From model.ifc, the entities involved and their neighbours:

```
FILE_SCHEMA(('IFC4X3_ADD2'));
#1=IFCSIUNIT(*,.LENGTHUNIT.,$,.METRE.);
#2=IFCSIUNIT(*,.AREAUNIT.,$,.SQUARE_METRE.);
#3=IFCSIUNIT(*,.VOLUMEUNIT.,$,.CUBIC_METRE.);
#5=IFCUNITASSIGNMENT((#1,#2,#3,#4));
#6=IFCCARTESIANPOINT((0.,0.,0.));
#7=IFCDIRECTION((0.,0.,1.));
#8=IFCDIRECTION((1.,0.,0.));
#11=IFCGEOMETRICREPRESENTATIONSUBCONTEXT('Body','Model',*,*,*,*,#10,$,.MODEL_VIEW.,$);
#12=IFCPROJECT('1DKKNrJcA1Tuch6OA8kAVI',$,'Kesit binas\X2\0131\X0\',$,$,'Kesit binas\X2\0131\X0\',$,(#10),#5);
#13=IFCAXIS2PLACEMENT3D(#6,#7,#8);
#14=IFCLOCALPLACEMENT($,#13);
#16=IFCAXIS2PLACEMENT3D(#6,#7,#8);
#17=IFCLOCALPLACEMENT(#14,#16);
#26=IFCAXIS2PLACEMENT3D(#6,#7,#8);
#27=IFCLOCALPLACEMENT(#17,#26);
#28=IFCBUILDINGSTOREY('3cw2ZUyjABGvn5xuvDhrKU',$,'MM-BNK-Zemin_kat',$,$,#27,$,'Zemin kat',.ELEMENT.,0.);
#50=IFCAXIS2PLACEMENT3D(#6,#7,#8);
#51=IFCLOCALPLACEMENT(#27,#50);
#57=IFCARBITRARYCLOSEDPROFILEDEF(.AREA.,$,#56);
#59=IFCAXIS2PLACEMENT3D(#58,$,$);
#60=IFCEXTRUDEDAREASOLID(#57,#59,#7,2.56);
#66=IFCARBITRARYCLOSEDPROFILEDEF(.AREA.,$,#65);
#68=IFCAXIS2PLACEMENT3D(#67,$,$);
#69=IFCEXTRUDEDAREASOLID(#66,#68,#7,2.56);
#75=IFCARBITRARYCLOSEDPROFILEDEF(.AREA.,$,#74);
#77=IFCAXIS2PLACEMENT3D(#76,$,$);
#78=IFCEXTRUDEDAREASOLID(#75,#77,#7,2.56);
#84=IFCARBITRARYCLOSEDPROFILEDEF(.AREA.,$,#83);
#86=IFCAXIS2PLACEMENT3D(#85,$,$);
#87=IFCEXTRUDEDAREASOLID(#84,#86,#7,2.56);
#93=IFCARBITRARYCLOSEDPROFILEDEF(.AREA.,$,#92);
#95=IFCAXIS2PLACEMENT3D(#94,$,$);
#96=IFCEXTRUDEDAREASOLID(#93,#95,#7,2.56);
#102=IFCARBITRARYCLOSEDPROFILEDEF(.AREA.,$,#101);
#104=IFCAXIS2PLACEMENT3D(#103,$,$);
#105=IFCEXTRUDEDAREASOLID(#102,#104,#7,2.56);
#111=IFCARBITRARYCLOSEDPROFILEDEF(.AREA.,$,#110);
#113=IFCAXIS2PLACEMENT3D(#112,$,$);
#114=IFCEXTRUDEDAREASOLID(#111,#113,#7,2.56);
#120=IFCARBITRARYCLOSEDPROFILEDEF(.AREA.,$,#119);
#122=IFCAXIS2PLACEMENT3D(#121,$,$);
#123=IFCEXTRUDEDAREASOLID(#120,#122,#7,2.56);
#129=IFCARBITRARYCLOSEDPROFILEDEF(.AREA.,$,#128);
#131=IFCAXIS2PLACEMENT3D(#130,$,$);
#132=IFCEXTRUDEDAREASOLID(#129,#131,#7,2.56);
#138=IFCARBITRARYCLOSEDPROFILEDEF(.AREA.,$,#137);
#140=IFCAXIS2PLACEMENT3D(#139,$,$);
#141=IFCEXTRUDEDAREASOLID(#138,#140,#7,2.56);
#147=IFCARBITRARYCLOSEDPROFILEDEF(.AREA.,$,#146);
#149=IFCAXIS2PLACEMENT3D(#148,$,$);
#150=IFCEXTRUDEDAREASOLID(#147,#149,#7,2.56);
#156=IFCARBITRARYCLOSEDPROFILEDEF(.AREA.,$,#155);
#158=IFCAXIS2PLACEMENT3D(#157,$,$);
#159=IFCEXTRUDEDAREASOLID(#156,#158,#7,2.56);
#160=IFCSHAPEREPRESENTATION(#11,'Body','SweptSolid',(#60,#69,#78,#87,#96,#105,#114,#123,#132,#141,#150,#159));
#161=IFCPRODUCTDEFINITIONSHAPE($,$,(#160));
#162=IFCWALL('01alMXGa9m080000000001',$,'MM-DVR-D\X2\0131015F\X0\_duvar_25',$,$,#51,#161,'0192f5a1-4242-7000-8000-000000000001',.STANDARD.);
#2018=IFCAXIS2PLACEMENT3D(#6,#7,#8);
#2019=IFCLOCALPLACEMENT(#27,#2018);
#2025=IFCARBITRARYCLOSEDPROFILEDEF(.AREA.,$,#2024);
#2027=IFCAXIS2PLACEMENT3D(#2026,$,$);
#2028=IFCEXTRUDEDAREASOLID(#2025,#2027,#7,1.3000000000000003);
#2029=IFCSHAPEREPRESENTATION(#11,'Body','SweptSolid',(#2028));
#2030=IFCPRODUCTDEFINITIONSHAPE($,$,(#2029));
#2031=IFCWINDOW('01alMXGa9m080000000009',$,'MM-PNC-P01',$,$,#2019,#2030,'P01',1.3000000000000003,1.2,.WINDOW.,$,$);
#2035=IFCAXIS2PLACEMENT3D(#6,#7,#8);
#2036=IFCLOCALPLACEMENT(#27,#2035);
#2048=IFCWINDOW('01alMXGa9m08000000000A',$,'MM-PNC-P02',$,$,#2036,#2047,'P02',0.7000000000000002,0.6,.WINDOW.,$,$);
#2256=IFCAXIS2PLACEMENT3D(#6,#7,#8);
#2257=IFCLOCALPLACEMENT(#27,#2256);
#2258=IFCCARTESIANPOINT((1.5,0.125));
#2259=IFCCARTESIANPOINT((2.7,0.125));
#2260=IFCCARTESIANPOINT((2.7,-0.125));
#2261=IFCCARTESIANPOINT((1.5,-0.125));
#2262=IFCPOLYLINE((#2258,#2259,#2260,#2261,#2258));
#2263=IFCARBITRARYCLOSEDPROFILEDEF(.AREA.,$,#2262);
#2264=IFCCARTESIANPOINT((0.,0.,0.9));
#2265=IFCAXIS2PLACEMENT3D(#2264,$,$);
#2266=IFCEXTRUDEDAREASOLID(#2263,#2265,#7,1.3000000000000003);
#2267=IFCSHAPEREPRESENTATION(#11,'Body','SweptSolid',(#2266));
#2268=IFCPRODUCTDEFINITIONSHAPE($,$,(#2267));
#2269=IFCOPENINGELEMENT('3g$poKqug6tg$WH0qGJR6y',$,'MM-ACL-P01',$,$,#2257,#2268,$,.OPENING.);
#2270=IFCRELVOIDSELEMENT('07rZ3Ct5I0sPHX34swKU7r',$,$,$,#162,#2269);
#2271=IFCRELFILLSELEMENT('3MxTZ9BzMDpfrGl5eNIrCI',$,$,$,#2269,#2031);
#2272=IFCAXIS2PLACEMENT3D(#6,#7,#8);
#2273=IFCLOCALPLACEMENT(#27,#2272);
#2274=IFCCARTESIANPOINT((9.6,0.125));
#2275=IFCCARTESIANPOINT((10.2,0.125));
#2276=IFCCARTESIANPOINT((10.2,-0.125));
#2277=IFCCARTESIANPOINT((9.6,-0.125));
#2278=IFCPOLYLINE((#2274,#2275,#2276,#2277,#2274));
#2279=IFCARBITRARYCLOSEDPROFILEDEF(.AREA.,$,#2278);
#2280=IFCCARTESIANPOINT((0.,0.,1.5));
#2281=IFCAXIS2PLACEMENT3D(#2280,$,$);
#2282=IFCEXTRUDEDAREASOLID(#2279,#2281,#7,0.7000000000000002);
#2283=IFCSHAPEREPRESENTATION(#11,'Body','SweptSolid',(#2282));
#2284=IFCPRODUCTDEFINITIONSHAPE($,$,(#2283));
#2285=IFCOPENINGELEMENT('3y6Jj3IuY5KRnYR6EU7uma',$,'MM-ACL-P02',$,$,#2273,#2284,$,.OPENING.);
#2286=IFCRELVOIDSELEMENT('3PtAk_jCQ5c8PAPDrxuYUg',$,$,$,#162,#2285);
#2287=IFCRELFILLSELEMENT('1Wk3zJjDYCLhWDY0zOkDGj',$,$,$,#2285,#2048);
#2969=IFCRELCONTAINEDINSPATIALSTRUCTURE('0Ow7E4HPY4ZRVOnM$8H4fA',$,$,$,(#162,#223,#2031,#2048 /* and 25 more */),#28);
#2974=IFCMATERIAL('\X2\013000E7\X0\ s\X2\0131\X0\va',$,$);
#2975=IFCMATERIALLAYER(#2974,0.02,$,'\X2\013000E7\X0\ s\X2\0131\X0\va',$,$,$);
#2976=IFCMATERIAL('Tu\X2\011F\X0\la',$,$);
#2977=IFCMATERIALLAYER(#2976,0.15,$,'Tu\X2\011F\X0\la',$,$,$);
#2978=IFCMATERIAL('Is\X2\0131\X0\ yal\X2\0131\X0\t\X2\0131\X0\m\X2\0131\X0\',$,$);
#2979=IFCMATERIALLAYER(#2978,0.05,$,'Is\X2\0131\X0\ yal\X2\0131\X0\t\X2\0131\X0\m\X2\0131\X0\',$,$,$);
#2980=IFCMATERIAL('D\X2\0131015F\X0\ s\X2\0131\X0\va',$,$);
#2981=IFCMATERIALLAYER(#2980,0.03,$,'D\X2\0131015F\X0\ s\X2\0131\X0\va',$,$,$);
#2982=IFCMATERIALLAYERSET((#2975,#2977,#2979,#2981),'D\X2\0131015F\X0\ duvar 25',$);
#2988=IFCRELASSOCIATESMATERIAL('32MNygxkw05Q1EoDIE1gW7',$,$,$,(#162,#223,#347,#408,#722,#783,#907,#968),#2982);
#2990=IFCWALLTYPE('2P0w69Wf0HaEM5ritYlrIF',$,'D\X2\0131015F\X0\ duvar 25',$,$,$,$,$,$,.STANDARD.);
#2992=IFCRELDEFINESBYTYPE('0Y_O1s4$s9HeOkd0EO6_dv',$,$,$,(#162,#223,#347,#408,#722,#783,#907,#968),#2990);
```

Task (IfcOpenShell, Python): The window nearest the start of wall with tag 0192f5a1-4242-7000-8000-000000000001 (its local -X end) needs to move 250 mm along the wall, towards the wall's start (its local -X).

```python
import ifcopenshell
import ifcopenshell.api.geometry
import ifcopenshell.util.placement

model = ifcopenshell.open("model.ifc")

window = model.by_guid("01alMXGa9m080000000009")
opening = window.FillsVoids[0].RelatingOpeningElement
wall = opening.VoidsElements[0].RelatingBuildingElement

wall_matrix = ifcopenshell.util.placement.get_local_placement(wall.ObjectPlacement)
shift = wall_matrix[:3, 0] * -0.25
before = ifcopenshell.util.placement.get_local_placement(window.ObjectPlacement)[:3, 3].copy()

# The window is not placed relative to its opening, so move both.
for product in (opening, window):
    matrix = ifcopenshell.util.placement.get_local_placement(product.ObjectPlacement)
    matrix[:3, 3] += shift
    ifcopenshell.api.geometry.edit_object_placement(model, product=product, matrix=matrix, is_si=False)

after = ifcopenshell.util.placement.get_local_placement(window.ObjectPlacement)[:3, 3]
print("window moved by", (after - before).round(3) + 0.0)

model.write("model_v2.ifc")
```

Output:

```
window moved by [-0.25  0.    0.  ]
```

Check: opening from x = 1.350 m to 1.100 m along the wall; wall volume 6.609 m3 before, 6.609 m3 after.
